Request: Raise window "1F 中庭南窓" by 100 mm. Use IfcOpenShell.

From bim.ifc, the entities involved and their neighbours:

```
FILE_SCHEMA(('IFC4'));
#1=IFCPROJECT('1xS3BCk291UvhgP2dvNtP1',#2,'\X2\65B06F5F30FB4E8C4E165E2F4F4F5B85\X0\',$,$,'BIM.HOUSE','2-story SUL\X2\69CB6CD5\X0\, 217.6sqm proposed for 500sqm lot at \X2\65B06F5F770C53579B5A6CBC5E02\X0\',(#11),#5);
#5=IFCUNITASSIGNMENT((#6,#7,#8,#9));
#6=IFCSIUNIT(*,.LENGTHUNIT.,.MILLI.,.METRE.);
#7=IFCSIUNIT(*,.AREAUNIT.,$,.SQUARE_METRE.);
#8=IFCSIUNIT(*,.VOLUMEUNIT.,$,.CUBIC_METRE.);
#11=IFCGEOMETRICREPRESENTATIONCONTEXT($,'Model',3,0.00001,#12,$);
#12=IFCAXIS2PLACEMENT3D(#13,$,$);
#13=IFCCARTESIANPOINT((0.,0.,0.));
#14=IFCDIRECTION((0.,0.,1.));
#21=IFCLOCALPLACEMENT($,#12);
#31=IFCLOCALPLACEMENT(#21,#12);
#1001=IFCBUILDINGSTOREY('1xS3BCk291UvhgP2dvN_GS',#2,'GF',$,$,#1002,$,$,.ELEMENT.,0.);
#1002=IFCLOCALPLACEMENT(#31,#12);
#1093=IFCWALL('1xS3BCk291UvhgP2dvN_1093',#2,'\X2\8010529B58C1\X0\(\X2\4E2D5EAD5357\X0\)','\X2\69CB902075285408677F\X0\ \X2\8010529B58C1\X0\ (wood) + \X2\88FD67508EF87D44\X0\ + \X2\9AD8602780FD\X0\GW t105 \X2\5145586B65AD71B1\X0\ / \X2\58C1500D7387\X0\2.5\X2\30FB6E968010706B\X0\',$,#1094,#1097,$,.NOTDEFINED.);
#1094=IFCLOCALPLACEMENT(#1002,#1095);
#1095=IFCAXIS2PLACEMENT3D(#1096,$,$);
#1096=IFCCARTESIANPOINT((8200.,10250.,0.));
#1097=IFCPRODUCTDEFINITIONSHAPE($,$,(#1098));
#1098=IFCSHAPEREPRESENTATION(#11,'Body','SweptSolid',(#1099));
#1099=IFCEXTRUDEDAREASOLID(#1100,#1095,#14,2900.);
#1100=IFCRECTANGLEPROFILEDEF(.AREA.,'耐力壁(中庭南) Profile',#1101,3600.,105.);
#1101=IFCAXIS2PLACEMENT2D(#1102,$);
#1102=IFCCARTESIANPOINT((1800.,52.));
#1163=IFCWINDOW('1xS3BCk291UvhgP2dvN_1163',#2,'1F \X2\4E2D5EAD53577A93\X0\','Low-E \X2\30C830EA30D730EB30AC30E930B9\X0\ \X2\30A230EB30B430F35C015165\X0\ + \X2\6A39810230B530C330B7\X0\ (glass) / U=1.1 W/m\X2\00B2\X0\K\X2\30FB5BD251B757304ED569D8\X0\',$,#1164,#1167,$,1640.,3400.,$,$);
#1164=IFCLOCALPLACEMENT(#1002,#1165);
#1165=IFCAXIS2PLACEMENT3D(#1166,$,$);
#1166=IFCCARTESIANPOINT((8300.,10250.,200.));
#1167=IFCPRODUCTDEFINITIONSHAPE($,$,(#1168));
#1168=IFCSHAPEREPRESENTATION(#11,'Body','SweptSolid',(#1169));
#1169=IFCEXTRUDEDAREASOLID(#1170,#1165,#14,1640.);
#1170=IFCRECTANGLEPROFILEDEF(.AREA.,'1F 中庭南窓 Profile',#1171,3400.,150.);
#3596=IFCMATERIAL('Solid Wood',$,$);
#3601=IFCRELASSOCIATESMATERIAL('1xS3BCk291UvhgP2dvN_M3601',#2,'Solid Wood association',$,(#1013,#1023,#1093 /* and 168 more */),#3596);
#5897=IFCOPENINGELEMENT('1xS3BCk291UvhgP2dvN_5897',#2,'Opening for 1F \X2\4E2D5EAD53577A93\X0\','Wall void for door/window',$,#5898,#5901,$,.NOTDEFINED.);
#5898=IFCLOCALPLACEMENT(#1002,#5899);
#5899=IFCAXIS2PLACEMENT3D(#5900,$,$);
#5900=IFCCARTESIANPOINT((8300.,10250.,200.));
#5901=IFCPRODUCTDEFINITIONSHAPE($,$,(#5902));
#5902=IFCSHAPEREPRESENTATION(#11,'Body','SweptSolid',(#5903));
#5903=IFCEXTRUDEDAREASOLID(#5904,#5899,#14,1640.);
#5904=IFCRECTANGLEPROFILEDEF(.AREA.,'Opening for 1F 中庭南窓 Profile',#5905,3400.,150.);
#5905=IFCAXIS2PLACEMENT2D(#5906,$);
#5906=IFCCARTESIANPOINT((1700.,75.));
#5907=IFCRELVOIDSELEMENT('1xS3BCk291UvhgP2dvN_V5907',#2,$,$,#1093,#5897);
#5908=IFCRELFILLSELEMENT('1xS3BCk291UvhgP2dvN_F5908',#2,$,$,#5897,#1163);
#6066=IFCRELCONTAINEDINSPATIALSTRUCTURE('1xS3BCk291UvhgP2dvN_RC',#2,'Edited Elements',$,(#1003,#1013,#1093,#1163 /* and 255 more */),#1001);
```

```python
import numpy as np
import ifcopenshell
import ifcopenshell.api.geometry
import ifcopenshell.util.placement
import ifcopenshell.util.unit

model = ifcopenshell.open("bim.ifc")
unit_scale = ifcopenshell.util.unit.calculate_unit_scale(model)

window = model.by_guid("1xS3BCk291UvhgP2dvN_1163")
opening = window.FillsVoids[0].RelatingOpeningElement
dz = 100.0

shift = np.array([0.0, 0.0, dz])
# The window is not placed relative to its opening, so move both.
for product in (opening, window):
    matrix = ifcopenshell.util.placement.get_local_placement(product.ObjectPlacement)
    matrix[:3, 3] += shift
    ifcopenshell.api.geometry.edit_object_placement(model, product=product, matrix=matrix, is_si=False)

print(f"moved by {dz * unit_scale:+.3f} m")

model.write("bim_rev.ifc")
```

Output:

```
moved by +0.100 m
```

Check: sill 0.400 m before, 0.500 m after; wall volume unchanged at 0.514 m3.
